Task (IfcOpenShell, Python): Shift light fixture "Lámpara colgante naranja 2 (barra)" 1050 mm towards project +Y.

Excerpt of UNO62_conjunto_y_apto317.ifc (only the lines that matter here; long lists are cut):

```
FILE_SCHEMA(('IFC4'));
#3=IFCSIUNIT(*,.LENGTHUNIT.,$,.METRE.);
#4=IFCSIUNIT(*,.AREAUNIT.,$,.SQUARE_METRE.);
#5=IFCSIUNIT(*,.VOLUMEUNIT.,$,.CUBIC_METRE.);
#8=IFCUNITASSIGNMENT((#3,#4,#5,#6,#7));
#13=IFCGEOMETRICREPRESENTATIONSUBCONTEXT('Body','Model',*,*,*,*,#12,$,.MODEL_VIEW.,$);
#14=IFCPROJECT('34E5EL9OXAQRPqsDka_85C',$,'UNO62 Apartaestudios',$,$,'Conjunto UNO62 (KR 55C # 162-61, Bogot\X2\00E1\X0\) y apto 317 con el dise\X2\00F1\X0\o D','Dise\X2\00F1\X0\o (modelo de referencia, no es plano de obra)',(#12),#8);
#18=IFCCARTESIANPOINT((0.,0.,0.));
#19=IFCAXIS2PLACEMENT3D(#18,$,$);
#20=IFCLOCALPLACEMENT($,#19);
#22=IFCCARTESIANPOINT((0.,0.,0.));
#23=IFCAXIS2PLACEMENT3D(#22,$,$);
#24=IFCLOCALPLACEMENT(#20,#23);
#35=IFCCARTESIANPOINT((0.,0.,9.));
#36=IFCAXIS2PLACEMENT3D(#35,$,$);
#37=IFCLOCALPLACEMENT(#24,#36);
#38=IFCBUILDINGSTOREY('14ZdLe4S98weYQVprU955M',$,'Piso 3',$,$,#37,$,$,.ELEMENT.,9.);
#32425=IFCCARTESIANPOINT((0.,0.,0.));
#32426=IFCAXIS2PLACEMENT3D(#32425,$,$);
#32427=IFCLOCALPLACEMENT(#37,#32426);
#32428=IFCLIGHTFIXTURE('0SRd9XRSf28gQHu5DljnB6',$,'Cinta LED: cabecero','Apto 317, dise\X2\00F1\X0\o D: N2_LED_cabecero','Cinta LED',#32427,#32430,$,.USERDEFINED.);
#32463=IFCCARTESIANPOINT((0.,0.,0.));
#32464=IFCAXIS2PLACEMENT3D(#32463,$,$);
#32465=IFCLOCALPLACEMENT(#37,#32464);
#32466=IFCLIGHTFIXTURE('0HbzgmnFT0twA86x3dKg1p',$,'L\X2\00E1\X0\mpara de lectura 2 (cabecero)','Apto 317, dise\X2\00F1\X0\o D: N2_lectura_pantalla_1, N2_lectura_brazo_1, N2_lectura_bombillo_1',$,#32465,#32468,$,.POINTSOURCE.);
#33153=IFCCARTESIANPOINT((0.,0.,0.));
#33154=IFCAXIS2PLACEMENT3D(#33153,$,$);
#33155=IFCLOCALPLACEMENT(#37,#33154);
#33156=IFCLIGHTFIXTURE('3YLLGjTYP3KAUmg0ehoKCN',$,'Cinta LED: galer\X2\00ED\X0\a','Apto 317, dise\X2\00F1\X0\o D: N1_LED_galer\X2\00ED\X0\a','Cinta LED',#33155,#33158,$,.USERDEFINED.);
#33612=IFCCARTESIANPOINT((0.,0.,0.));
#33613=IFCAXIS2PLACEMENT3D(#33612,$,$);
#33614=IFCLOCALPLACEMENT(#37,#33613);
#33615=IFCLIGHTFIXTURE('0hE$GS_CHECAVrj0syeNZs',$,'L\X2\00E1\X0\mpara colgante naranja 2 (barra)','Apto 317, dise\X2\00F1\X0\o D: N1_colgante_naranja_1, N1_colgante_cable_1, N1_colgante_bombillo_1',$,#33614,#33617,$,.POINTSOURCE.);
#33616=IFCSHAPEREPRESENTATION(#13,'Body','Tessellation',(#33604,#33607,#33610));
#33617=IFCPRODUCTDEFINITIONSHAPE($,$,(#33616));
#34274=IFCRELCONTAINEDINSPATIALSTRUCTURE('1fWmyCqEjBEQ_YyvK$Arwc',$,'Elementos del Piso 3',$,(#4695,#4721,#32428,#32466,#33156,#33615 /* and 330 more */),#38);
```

```python
import ifcopenshell
import ifcopenshell.api.geometry
import ifcopenshell.util.placement
import ifcopenshell.util.unit

model = ifcopenshell.open("UNO62_conjunto_y_apto317.ifc")
unit_scale = ifcopenshell.util.unit.calculate_unit_scale(model)

item = model.by_guid("0hE$GS_CHECAVrj0syeNZs")
matrix = ifcopenshell.util.placement.get_local_placement(item.ObjectPlacement)
matrix[1, 3] += 1.05 / unit_scale
ifcopenshell.api.geometry.edit_object_placement(model, product=item, matrix=matrix, is_si=False)

print(ifcopenshell.util.placement.get_local_placement(item.ObjectPlacement).round(3) + 0.0)

model.write("UNO62_conjunto_y_apto317_rev.ifc")
```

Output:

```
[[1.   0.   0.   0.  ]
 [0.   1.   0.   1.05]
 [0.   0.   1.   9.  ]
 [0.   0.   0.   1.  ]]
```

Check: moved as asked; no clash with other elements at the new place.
